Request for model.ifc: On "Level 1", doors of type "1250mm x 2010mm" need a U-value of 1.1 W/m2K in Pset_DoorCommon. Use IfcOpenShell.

First a look at what the model holds.

```python
import ifcopenshell
import ifcopenshell.util.element

model = ifcopenshell.open("model.ifc")
print(model.schema)
storey = next(s for s in model.by_type("IfcBuildingStorey") if s.Name == "Level 1")
doors = [e for e in ifcopenshell.util.element.get_decomposition(storey) if e.is_a("IfcDoor")]
seen = {}
for e in doors:
    element_type = ifcopenshell.util.element.get_type(e)
    key = (element_type.Name if element_type != e and element_type else None, ifcopenshell.util.element.get_pset(e, "Pset_DoorCommon", "ThermalTransmittance"))
    seen[key] = seen.get(key, 0) + 1
for (name, value), count in sorted(seen.items(), key=str):
    print(count, "x", name, "|", value)
```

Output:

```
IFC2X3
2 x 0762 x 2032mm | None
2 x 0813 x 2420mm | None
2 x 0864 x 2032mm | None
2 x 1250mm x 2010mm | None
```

```python
import ifcopenshell
import ifcopenshell.api.pset
import ifcopenshell.util.element

model = ifcopenshell.open("model.ifc")

storey = next(s for s in model.by_type("IfcBuildingStorey") if s.Name == "Level 1")
doors = [e for e in ifcopenshell.util.element.get_decomposition(storey) if e.is_a("IfcDoor")]

count = 0
for e in doors:
    element_type = ifcopenshell.util.element.get_type(e)
    if element_type in (None, e) or element_type.Name != "1250mm x 2010mm":
        continue
    # add_pset returns the element's existing set when there is one.
    pset = ifcopenshell.api.pset.add_pset(model, product=e, name="Pset_DoorCommon")
    ifcopenshell.api.pset.edit_pset(model, pset=pset, properties={"ThermalTransmittance": 1.1})
    count += 1

print(count, "doors updated")

model.write("model_rev.ifc")
```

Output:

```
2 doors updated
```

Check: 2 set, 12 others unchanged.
